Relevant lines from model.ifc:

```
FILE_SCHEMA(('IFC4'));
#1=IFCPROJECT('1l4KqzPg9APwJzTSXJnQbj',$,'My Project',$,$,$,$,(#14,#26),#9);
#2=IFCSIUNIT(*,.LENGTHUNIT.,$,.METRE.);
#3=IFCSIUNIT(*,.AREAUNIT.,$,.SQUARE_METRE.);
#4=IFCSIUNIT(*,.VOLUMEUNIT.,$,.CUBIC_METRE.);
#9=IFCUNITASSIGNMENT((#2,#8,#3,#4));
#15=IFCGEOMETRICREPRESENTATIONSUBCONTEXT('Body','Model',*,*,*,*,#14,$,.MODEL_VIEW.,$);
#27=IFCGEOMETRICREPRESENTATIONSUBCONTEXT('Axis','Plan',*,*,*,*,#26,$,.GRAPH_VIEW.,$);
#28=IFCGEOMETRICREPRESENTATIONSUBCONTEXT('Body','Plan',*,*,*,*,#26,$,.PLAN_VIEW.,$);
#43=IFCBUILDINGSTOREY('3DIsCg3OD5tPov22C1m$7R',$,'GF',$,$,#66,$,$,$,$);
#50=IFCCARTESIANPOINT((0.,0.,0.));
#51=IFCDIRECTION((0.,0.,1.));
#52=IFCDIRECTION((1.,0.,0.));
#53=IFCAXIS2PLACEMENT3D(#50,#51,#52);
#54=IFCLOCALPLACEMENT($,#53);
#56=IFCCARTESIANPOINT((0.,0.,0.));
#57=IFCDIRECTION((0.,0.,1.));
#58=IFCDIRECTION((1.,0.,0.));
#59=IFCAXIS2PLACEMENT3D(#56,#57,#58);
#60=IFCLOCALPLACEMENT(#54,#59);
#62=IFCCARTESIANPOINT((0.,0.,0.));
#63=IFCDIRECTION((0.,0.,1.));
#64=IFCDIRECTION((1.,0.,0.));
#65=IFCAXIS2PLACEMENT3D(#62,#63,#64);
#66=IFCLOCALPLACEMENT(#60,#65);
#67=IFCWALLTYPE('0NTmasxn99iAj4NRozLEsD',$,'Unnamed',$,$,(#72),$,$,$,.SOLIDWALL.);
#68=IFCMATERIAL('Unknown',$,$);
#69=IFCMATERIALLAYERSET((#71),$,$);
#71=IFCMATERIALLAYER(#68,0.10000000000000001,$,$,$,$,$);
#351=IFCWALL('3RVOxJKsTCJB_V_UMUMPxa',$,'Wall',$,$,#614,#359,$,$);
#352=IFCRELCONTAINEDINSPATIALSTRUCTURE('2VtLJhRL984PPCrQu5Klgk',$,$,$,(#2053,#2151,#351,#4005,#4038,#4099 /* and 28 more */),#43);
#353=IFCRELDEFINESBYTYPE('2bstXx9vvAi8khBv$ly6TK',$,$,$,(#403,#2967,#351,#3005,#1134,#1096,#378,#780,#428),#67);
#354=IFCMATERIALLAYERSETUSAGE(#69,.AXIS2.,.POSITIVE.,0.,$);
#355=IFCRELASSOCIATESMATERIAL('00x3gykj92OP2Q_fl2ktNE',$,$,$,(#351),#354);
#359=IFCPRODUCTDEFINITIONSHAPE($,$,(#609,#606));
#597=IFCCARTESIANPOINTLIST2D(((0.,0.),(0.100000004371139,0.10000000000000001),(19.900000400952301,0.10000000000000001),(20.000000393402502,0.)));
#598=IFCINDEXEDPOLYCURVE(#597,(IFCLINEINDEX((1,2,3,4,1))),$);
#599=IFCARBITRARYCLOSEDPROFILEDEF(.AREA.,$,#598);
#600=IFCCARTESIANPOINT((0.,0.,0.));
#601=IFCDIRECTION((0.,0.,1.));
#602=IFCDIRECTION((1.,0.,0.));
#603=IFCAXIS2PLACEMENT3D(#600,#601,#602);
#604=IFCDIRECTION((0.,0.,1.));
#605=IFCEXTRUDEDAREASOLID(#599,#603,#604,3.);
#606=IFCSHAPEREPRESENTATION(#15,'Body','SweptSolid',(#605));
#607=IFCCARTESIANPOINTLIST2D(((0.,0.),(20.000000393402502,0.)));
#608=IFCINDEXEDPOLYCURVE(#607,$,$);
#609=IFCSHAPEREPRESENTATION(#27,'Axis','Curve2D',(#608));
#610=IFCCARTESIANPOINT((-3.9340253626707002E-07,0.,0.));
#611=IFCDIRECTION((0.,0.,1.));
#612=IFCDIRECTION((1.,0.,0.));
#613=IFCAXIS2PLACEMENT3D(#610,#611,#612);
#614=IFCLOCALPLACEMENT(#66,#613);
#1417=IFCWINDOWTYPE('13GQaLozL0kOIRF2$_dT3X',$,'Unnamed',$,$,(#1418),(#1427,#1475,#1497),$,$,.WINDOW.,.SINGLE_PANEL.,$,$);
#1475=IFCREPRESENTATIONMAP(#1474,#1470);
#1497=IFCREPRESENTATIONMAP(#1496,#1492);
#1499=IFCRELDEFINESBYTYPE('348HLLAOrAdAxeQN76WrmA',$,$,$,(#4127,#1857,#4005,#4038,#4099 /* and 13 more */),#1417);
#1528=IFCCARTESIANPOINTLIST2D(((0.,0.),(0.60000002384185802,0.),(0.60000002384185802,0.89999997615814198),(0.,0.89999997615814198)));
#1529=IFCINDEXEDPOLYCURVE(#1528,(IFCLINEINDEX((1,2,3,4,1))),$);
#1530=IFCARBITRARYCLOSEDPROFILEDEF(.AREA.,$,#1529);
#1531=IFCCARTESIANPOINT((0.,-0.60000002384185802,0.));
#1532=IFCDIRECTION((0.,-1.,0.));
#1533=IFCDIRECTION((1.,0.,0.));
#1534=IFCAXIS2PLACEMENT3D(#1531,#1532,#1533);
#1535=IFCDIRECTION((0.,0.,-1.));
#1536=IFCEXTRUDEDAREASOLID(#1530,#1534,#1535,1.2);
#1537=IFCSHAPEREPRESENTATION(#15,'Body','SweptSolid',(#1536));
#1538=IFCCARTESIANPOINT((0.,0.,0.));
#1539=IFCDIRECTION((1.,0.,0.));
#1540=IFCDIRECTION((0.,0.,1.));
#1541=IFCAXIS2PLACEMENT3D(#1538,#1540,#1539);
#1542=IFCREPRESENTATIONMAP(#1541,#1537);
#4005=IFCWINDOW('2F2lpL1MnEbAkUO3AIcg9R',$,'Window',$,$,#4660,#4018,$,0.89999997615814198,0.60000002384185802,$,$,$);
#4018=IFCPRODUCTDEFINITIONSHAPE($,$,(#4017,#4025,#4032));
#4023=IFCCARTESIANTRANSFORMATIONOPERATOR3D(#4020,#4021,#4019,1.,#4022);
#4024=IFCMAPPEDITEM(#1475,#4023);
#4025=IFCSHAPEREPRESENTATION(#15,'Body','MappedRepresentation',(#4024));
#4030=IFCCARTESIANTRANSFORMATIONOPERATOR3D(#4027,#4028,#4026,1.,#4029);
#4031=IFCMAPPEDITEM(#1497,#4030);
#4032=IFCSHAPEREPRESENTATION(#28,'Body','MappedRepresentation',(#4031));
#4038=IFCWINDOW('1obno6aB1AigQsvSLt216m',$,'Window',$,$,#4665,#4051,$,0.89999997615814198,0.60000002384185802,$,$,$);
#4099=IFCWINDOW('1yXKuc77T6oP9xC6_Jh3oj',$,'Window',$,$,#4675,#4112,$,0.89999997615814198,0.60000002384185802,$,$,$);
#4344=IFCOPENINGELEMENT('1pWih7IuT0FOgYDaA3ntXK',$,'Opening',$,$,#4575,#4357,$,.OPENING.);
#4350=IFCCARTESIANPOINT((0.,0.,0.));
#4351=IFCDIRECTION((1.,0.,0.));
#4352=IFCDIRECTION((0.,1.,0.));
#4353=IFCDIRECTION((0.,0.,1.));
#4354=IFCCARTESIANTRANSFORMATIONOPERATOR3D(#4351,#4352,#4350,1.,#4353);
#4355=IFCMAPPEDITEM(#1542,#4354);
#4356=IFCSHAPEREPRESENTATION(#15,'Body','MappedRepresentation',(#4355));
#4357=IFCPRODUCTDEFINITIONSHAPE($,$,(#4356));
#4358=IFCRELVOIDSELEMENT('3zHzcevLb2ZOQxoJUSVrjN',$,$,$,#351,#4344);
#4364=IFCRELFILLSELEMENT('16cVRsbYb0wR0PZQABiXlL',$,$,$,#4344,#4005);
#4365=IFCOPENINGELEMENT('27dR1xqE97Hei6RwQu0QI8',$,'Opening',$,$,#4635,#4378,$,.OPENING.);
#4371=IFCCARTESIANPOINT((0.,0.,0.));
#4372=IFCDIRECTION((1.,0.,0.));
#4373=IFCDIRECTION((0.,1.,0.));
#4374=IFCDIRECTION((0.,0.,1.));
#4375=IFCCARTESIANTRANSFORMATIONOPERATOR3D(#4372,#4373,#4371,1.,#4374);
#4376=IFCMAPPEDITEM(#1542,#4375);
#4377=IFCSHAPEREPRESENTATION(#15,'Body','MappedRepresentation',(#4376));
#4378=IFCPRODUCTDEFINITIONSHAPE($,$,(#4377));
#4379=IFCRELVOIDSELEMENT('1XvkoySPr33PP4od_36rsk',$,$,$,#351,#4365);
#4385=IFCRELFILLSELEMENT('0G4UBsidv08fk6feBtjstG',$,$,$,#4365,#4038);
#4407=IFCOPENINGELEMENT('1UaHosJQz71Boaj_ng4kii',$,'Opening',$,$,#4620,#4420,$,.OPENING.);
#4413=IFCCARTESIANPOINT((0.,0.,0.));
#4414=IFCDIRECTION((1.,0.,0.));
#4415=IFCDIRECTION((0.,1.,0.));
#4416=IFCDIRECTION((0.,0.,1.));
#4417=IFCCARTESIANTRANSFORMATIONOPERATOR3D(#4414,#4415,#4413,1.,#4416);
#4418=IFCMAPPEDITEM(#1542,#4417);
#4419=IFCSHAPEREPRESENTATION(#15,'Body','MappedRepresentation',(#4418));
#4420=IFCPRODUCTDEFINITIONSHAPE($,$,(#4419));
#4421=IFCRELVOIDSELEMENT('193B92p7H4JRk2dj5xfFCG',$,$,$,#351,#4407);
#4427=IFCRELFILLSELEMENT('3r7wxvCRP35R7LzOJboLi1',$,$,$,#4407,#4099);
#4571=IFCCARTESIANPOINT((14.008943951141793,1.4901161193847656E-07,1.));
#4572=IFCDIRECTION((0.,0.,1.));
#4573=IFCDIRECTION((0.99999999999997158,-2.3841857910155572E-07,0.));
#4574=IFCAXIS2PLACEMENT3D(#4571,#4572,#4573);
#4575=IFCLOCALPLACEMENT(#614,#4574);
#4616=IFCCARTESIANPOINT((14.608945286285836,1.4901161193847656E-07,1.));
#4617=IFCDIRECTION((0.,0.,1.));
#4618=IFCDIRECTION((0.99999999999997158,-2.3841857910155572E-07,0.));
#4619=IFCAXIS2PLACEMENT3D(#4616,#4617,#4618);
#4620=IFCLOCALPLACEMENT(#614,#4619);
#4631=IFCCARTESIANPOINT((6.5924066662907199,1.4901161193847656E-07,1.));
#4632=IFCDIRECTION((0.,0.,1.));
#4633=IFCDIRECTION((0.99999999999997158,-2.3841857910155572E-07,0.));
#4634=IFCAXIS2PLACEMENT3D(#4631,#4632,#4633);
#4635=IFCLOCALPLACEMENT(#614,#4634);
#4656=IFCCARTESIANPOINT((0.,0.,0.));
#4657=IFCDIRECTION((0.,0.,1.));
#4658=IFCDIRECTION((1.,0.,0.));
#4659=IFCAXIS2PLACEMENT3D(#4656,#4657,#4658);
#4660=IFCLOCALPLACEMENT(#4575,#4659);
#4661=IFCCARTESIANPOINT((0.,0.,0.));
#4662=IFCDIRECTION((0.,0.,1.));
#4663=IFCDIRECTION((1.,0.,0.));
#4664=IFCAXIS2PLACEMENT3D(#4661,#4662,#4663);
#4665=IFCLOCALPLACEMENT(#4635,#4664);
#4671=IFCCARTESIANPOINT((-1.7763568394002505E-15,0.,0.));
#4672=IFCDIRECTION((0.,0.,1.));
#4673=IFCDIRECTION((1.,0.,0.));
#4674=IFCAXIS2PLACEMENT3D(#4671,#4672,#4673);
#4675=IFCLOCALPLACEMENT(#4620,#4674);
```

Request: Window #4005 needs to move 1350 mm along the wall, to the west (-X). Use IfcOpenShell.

```python
import ifcopenshell
import ifcopenshell.api.geometry
import ifcopenshell.util.placement

model = ifcopenshell.open("model.ifc")

window = model.by_guid("2F2lpL1MnEbAkUO3AIcg9R")
opening = window.FillsVoids[0].RelatingOpeningElement
wall = opening.VoidsElements[0].RelatingBuildingElement

wall_matrix = ifcopenshell.util.placement.get_local_placement(wall.ObjectPlacement)
shift = wall_matrix[:3, 0] * -1.35
before = ifcopenshell.util.placement.get_local_placement(window.ObjectPlacement)[:3, 3].copy()

# The window is placed relative to its opening, so it follows when the opening moves.
matrix = ifcopenshell.util.placement.get_local_placement(opening.ObjectPlacement)
matrix[:3, 3] += shift
ifcopenshell.api.geometry.edit_object_placement(
    model, product=opening, matrix=matrix, is_si=False, should_transform_children=True
)

after = ifcopenshell.util.placement.get_local_placement(window.ObjectPlacement)[:3, 3]
print("window moved by", (after - before).round(3) + 0.0)

model.write("model-out.ifc")
```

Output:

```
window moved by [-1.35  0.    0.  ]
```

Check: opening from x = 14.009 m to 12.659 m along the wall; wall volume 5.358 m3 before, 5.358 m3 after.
